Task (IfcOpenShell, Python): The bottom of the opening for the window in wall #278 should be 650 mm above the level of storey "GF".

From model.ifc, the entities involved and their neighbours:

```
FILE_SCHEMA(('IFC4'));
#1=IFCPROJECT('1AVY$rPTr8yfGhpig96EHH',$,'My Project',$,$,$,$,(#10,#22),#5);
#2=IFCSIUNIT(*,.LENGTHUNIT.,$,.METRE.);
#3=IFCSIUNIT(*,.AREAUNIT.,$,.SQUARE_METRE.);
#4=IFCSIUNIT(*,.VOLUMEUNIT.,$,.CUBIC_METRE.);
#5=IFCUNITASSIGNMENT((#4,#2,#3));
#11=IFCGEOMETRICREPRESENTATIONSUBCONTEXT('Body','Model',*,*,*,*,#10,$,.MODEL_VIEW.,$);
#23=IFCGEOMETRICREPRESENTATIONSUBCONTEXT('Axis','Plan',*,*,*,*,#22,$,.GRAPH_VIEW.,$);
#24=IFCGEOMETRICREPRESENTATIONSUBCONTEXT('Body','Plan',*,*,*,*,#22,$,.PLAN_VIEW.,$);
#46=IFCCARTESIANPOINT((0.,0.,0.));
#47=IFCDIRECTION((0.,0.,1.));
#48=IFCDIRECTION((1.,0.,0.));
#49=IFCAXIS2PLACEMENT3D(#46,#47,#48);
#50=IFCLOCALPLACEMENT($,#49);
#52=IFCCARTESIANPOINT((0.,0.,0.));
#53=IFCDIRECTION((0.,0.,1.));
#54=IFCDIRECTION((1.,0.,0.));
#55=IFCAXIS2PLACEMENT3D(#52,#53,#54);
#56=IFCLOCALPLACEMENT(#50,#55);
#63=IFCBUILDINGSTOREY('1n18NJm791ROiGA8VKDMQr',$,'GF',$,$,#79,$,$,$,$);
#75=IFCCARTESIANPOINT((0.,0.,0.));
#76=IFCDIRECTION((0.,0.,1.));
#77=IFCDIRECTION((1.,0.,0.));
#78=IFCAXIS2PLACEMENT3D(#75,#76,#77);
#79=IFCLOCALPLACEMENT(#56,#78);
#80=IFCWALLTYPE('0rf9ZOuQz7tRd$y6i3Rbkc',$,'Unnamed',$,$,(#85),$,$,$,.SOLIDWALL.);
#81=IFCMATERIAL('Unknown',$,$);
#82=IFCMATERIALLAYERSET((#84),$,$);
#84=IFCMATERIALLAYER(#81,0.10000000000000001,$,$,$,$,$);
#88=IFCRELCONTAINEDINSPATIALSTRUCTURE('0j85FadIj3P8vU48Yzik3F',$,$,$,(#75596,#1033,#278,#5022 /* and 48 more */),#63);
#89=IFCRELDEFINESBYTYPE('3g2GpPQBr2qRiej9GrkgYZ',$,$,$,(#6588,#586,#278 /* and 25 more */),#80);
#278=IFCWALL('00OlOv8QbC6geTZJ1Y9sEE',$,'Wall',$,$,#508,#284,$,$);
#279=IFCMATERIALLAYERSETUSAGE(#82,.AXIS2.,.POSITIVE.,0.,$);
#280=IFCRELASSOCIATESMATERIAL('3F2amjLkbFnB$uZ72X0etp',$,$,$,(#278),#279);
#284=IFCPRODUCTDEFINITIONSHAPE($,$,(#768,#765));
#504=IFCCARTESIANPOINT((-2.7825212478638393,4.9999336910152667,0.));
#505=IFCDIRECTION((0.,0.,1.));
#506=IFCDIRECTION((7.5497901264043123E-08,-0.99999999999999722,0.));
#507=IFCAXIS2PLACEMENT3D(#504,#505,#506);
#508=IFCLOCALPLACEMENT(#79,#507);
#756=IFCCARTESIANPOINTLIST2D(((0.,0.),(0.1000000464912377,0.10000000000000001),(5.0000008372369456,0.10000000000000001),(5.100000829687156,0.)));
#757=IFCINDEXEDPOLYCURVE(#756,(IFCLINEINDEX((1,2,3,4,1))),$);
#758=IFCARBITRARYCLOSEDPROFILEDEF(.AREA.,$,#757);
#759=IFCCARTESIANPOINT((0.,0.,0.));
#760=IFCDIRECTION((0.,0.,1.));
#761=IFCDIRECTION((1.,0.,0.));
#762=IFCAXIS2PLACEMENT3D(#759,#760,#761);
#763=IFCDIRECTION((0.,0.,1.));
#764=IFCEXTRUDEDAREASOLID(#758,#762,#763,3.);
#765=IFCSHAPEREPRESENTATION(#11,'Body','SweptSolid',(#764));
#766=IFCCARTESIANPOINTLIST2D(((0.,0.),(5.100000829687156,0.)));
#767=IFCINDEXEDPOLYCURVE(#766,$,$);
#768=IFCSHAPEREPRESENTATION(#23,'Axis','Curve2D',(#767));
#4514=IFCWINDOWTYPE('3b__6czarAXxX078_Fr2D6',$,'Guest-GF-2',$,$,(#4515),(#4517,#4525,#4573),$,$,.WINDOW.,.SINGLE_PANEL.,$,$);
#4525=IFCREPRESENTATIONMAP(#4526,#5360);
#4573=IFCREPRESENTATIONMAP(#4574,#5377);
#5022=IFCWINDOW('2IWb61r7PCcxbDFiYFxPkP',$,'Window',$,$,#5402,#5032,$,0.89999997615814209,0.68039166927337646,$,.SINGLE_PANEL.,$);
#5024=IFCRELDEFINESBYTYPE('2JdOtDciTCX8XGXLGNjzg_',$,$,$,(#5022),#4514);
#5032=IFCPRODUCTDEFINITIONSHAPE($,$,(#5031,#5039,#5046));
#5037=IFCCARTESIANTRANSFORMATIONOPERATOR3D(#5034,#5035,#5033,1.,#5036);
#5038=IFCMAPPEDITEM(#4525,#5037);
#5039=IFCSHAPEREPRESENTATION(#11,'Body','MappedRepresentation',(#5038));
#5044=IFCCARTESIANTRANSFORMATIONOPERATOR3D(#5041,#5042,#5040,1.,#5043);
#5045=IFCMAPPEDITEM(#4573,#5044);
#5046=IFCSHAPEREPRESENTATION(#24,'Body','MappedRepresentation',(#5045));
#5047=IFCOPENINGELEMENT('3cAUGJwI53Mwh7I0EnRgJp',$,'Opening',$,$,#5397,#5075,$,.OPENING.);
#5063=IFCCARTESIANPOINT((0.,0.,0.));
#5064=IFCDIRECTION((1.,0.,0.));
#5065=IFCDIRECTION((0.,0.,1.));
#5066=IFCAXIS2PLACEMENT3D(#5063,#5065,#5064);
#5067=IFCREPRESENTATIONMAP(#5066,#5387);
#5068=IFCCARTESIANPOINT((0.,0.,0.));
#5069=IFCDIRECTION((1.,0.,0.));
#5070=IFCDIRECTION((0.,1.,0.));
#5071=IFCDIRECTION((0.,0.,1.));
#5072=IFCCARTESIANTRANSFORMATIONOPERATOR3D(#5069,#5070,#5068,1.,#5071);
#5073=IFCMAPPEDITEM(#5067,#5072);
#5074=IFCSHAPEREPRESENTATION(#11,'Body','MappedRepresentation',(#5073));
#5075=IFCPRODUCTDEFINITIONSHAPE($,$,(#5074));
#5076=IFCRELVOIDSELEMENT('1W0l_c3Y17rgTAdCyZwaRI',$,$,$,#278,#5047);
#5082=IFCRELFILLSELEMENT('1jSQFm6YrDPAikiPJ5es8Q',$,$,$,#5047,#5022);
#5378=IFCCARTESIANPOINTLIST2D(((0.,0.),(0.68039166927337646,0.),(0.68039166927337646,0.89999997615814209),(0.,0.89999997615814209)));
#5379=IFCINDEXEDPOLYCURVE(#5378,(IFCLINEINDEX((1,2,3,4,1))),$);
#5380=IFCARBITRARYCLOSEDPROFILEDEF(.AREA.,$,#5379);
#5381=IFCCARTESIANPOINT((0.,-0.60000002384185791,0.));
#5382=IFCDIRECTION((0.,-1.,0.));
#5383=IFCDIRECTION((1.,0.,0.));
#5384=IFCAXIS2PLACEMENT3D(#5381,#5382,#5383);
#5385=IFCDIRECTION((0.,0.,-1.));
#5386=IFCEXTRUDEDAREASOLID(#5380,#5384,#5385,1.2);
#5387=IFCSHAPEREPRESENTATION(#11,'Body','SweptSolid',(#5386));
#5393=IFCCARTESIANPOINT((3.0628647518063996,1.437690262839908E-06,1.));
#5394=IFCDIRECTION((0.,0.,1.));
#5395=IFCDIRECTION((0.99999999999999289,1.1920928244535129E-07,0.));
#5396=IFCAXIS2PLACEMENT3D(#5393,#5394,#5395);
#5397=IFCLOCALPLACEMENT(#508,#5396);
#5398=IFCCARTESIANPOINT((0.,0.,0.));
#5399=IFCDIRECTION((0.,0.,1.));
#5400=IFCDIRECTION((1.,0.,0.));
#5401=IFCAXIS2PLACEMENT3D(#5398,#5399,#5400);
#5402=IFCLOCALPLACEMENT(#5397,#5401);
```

```python
import numpy as np
import ifcopenshell
import ifcopenshell.api.geometry
import ifcopenshell.geom
import ifcopenshell.util.element
import ifcopenshell.util.placement
import ifcopenshell.util.shape
import ifcopenshell.util.unit

model = ifcopenshell.open("model.ifc")
unit_scale = ifcopenshell.util.unit.calculate_unit_scale(model)

window = model.by_guid("2IWb61r7PCcxbDFiYFxPkP")
opening = window.FillsVoids[0].RelatingOpeningElement
storey = ifcopenshell.util.element.get_container(window, ifc_class="IfcBuildingStorey")
level = ifcopenshell.util.placement.get_local_placement(storey.ObjectPlacement)[2, 3]

# The opening's origin need not be at the sill, so measure its lowest point.
shape = ifcopenshell.geom.create_shape(ifcopenshell.geom.settings(), opening)
bottom = ifcopenshell.util.shape.get_shape_bottom_elevation(shape, shape.geometry) / unit_scale
dz = level + 0.65 - bottom

shift = np.array([0.0, 0.0, dz])
# The window is placed relative to its opening, so it follows when the opening moves.
matrix = ifcopenshell.util.placement.get_local_placement(opening.ObjectPlacement)
matrix[:3, 3] += shift
ifcopenshell.api.geometry.edit_object_placement(
    model, product=opening, matrix=matrix, is_si=False, should_transform_children=True
)

print(f"moved by {dz * unit_scale:+.3f} m")

model.write("model_updated.ifc")
```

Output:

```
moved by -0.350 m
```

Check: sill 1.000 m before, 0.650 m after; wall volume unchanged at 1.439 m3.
